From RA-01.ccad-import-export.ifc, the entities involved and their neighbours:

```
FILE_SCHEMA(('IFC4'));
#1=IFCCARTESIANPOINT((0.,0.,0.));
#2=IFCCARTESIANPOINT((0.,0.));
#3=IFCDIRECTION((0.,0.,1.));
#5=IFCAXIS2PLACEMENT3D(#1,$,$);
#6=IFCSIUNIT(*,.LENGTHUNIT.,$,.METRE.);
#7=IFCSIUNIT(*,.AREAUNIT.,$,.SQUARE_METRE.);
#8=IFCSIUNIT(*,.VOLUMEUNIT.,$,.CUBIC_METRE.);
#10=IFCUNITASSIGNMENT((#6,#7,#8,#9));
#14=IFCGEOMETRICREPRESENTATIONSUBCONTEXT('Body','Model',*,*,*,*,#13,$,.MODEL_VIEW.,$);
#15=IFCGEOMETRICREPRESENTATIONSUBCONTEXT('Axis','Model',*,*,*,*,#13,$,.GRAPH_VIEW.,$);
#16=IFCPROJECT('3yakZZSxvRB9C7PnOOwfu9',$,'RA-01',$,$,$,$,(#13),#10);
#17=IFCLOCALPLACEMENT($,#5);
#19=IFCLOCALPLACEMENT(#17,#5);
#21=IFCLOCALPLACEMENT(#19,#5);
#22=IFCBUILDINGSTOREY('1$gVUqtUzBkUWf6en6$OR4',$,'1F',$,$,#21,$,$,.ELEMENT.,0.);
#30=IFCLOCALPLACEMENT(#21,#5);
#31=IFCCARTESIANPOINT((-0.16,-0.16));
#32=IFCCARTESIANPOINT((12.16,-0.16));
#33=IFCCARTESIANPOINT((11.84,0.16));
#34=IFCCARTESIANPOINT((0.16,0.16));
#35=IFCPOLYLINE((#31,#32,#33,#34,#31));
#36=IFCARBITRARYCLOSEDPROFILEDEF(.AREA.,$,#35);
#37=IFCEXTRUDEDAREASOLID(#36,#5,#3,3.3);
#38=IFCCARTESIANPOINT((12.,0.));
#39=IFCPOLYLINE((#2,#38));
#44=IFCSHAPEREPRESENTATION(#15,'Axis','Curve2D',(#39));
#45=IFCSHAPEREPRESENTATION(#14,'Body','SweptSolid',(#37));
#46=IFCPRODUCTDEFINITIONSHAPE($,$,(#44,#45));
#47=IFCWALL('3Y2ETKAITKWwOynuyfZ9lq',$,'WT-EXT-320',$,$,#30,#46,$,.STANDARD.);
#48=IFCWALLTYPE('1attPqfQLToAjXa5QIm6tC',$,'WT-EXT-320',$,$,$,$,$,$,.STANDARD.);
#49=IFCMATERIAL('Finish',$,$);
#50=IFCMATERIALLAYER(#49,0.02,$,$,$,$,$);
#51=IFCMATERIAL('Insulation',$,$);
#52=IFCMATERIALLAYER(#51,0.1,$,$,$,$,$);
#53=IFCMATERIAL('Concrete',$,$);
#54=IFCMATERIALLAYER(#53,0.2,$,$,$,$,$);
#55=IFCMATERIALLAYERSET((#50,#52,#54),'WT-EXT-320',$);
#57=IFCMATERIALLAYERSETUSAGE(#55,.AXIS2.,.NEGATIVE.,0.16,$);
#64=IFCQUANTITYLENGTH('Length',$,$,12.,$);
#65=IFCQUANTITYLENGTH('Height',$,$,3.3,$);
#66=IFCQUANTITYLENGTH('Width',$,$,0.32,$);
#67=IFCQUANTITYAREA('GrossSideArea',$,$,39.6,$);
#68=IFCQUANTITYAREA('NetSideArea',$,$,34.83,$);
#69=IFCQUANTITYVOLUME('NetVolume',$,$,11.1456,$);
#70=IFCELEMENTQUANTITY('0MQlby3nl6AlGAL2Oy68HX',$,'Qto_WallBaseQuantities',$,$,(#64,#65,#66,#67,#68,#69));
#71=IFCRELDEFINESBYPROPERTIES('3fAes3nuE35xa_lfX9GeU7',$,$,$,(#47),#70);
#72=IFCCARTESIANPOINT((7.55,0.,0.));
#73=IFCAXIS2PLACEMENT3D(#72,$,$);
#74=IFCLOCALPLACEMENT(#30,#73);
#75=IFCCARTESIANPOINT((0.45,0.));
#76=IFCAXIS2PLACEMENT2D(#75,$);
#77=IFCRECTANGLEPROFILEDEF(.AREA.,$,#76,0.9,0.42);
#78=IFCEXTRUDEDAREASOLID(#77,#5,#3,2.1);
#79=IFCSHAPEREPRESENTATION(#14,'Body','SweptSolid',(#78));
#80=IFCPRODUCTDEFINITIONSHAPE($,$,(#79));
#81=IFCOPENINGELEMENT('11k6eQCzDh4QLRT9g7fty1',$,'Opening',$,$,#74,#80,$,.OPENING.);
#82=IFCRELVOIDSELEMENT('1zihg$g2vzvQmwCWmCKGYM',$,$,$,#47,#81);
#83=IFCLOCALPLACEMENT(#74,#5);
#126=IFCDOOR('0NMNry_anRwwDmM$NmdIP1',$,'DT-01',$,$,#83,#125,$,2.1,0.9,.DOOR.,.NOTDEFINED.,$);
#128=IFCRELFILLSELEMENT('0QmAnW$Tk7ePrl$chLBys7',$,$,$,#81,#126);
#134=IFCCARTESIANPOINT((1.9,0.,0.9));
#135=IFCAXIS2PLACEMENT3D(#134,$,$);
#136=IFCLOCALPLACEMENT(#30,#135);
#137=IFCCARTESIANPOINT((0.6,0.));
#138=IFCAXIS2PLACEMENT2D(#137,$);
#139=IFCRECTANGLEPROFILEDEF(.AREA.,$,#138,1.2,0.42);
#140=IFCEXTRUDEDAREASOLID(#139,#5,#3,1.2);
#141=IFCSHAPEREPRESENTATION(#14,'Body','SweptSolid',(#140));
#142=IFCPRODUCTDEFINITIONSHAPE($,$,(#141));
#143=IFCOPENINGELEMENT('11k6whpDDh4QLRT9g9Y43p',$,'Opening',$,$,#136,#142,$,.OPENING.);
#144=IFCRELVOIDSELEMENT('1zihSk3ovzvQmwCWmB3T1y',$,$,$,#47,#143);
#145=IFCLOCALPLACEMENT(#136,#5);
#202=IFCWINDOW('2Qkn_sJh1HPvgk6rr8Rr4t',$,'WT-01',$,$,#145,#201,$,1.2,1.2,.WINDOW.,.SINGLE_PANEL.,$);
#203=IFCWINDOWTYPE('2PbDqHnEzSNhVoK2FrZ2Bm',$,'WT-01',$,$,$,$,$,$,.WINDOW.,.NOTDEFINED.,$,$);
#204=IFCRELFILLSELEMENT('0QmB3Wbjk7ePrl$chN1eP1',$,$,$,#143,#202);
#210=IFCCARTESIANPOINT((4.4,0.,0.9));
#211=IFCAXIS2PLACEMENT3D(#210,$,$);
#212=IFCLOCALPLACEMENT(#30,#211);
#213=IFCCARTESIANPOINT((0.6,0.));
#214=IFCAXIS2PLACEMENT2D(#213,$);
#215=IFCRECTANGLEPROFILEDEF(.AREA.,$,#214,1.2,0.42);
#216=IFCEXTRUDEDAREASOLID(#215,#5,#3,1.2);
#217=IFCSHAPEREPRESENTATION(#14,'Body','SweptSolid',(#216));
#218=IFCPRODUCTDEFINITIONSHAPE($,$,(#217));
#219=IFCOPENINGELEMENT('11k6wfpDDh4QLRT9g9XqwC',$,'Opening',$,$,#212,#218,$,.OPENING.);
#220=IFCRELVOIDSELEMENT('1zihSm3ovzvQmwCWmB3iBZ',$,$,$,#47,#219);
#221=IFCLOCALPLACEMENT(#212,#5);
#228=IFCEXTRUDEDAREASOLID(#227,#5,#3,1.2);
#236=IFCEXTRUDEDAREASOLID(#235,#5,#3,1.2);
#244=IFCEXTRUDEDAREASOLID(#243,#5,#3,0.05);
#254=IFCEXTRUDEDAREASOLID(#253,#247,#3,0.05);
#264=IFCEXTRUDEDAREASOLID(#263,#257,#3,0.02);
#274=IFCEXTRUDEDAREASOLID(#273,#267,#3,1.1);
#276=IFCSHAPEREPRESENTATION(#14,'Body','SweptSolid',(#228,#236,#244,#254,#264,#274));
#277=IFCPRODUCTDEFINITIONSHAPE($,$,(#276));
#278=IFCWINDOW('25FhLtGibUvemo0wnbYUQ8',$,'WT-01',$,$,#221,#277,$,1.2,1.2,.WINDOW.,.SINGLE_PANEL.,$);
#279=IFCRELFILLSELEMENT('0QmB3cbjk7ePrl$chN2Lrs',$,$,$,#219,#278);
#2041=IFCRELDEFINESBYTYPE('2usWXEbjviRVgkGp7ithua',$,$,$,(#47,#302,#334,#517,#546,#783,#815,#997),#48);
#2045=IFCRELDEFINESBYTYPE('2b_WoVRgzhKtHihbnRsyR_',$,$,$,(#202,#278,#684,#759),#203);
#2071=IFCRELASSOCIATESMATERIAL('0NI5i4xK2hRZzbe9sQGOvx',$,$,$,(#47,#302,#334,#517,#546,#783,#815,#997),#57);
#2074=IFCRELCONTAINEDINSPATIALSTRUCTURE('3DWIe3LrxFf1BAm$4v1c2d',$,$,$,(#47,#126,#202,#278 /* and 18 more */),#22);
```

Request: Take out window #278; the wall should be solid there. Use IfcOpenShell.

```python
import ifcopenshell
import ifcopenshell.api.feature
import ifcopenshell.api.pset
import ifcopenshell.api.root
import ifcopenshell.geom
import ifcopenshell.util.element
import ifcopenshell.util.shape
import ifcopenshell.util.unit

model = ifcopenshell.open("RA-01.ccad-import-export.ifc")
area_scale = ifcopenshell.util.unit.calculate_unit_scale(model, "AREAUNIT")
volume_scale = ifcopenshell.util.unit.calculate_unit_scale(model, "VOLUMEUNIT")
settings = ifcopenshell.geom.settings()


def volume(element):
    """Net volume in cubic metres, openings subtracted."""
    shape = ifcopenshell.geom.create_shape(settings, element)
    return ifcopenshell.util.shape.get_volume(shape.geometry)


window = model.by_id(278)
opening = window.FillsVoids[0].RelatingOpeningElement
wall = opening.VoidsElements[0].RelatingBuildingElement
before = volume(wall)

ifcopenshell.api.root.remove_product(model, product=window)
ifcopenshell.api.feature.remove_feature(model, feature=opening)

after = volume(wall)
thickness = 0.32  # wall thickness in metres

# Update the wall's stored quantities.
qto = model.by_id(ifcopenshell.util.element.get_pset(wall, "Qto_WallBaseQuantities", should_inherit=False)["id"])
ifcopenshell.api.pset.edit_qto(model, qto=qto, properties={
    "NetSideArea": after / thickness / area_scale,
    "NetVolume": after / volume_scale,
})

print(f"wall volume {before:.3f} -> {after:.3f} m3")

model.write("RA-01.ccad-import-export_updated.ifc")
```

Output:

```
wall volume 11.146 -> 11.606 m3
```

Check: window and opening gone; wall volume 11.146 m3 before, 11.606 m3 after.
